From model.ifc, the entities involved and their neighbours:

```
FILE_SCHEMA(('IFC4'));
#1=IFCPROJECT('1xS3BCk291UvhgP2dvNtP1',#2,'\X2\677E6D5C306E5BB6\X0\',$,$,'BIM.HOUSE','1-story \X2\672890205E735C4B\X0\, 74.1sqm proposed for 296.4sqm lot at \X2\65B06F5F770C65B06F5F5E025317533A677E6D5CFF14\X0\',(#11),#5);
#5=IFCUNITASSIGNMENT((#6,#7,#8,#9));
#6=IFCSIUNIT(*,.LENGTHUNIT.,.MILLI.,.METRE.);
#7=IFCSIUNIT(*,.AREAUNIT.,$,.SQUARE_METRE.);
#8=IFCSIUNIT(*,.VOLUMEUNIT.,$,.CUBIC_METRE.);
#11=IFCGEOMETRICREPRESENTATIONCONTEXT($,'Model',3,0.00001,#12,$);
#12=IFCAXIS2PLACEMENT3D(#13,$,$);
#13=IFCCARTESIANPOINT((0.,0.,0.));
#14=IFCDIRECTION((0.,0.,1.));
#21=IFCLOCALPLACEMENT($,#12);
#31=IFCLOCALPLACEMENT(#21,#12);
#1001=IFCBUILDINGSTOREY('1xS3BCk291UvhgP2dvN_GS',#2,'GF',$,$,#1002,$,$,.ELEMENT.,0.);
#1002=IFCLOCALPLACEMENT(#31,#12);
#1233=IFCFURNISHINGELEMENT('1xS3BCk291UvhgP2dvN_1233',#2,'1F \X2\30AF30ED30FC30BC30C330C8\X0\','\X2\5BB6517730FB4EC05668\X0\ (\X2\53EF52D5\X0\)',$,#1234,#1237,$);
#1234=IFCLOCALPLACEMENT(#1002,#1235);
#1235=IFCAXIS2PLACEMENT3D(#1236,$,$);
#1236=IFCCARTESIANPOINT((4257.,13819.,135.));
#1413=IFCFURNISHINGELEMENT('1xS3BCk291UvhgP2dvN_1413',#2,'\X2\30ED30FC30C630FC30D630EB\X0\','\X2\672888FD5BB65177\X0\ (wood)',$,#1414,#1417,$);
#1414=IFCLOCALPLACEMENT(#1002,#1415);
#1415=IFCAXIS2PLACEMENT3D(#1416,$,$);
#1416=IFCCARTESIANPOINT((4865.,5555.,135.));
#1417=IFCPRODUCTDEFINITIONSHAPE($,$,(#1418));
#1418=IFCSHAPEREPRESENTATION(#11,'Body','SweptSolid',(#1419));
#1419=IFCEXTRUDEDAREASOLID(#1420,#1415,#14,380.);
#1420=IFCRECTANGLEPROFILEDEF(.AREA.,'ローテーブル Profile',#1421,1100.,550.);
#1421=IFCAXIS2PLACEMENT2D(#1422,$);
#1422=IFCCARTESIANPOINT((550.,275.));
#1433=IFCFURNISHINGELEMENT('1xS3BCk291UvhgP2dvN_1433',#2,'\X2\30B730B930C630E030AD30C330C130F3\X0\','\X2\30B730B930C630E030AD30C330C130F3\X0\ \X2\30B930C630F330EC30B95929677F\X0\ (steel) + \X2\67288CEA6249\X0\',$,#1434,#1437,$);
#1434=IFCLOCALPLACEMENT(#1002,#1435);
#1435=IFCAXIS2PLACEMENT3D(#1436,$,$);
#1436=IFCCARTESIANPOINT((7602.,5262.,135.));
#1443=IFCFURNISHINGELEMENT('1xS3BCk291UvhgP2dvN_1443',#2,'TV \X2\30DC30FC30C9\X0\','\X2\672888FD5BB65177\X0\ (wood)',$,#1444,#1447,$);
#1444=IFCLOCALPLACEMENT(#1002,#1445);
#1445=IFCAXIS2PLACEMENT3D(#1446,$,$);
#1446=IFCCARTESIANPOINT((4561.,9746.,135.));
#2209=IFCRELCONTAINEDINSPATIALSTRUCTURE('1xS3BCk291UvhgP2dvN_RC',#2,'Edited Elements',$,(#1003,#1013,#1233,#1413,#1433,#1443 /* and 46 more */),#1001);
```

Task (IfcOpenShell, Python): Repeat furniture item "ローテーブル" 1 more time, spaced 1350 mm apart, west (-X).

```python
import numpy as np
import ifcopenshell
import ifcopenshell.api.geometry
import ifcopenshell.api.root
import ifcopenshell.util.element
import ifcopenshell.util.placement
import ifcopenshell.util.unit

model = ifcopenshell.open("model.ifc")
unit_scale = ifcopenshell.util.unit.calculate_unit_scale(model)


def reuse_history(source, copy):
    """copy_class also copies each property set's owner history, people and application; keep the originals."""
    for rel in copy.IsDefinedBy:
        if rel.is_a("IfcRelDefinesByProperties") and (history := rel.RelatingPropertyDefinition.OwnerHistory):
            rel.RelatingPropertyDefinition.OwnerHistory = source.OwnerHistory
            ifcopenshell.util.element.remove_deep2(model, history)


source = model.by_guid("1xS3BCk291UvhgP2dvN_1413")
base = ifcopenshell.util.placement.get_local_placement(source.ObjectPlacement)
step = np.array([-1.0, 0.0, 0.0]) * 1.35 / unit_scale

for i in range(1, 2):
    copy = ifcopenshell.api.root.copy_class(model, product=source)
    copy.Representation = ifcopenshell.util.element.copy_deep(
        model, source.Representation, exclude=["IfcGeometricRepresentationContext", "IfcRepresentationMap"]
    )
    reuse_history(source, copy)
    matrix = base.copy()
    matrix[:3, 3] += i * step
    print("added at", matrix[:3, 3].round(3) + 0.0)
    ifcopenshell.api.geometry.edit_object_placement(model, product=copy, matrix=matrix, is_si=False)

model.write("model-out.ifc")
```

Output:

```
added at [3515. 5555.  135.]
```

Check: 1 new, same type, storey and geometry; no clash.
